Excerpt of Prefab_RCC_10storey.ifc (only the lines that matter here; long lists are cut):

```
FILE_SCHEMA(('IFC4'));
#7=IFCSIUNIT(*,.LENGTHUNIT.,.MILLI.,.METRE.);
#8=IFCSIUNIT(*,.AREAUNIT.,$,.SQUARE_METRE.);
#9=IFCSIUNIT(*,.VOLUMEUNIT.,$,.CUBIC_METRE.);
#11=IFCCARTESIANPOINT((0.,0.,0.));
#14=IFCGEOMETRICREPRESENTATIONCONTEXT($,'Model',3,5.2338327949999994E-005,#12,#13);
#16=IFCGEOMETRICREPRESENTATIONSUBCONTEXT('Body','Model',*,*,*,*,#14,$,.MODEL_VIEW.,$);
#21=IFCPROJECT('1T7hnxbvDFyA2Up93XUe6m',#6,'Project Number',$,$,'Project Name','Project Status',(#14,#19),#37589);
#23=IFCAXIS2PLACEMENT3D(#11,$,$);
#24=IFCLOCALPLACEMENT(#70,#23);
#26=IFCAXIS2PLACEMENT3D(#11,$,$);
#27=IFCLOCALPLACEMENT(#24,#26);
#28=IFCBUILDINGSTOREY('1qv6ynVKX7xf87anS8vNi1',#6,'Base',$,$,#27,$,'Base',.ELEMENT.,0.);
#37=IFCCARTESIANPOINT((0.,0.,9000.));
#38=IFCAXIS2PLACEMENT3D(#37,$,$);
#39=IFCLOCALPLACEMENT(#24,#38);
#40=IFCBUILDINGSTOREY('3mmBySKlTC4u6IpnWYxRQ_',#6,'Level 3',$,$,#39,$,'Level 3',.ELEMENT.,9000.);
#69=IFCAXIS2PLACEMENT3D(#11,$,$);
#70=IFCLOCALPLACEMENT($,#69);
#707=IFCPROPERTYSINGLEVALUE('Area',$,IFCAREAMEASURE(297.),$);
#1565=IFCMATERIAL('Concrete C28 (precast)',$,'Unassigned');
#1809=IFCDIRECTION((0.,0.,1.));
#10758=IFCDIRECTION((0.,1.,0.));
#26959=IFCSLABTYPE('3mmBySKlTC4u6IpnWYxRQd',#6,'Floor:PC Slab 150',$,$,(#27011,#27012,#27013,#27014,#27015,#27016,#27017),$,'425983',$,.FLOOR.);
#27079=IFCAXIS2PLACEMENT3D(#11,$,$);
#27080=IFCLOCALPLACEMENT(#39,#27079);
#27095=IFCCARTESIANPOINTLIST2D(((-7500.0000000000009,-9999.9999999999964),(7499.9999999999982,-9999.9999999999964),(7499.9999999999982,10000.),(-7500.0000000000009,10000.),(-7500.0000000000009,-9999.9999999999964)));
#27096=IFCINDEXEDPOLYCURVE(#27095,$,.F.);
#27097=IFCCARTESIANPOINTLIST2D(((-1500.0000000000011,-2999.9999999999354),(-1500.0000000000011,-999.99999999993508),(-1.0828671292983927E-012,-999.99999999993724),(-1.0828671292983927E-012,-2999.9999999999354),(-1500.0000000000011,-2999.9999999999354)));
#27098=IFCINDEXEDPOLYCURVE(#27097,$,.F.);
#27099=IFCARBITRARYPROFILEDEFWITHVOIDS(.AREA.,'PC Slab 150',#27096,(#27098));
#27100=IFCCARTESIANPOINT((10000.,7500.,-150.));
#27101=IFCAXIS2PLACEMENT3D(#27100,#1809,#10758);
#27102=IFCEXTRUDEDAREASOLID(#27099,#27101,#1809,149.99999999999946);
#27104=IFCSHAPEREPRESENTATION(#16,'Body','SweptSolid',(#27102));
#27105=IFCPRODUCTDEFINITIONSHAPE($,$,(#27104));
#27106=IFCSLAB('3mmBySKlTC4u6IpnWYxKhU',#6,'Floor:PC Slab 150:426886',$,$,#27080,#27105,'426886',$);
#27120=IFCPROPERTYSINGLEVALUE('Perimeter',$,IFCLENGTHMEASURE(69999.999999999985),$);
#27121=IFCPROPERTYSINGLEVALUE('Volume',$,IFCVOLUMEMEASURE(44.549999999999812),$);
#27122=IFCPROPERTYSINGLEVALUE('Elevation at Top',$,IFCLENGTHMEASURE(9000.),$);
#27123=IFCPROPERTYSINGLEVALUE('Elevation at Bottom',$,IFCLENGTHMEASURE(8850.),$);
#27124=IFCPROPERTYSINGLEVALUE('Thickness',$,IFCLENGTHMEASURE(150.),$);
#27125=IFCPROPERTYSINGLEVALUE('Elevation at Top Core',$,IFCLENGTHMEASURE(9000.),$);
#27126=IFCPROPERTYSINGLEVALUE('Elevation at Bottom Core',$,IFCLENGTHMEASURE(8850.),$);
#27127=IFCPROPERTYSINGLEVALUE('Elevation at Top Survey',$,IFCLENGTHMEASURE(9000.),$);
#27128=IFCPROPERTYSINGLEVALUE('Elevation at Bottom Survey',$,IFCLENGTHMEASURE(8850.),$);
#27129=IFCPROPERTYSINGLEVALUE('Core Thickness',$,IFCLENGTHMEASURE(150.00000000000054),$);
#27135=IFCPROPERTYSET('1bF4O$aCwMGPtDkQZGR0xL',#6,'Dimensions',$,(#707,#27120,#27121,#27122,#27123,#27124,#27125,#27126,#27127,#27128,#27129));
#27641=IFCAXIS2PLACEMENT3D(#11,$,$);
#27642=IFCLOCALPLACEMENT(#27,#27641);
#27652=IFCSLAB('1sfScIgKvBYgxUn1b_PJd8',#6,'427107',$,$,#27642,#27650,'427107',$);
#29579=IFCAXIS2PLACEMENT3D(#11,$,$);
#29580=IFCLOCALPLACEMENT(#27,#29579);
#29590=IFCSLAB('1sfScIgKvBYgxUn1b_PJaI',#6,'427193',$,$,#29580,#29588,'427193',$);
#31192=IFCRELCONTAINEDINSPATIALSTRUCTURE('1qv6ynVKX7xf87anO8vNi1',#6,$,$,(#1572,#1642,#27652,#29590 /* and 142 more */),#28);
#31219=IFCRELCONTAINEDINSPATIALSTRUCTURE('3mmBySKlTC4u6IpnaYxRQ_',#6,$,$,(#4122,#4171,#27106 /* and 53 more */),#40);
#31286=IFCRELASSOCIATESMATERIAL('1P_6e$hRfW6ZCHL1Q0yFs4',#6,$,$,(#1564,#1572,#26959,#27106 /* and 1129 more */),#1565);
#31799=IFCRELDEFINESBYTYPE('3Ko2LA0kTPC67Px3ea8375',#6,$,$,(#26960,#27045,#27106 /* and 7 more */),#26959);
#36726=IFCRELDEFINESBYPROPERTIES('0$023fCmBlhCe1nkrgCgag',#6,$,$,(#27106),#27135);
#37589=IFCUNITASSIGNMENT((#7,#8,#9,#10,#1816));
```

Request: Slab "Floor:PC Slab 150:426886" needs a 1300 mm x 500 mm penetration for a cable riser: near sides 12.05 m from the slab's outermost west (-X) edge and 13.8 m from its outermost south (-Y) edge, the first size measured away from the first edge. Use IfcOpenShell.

```python
import numpy as np
import ifcopenshell
import ifcopenshell.api.feature
import ifcopenshell.api.geometry
import ifcopenshell.api.pset
import ifcopenshell.api.root
import ifcopenshell.geom
import ifcopenshell.util.element
import ifcopenshell.util.placement
import ifcopenshell.util.representation
import ifcopenshell.util.shape
import ifcopenshell.util.unit

model = ifcopenshell.open("Prefab_RCC_10storey.ifc")
unit_scale = ifcopenshell.util.unit.calculate_unit_scale(model)
area_scale = ifcopenshell.util.unit.calculate_unit_scale(model, "AREAUNIT")
volume_scale = ifcopenshell.util.unit.calculate_unit_scale(model, "VOLUMEUNIT")
settings = ifcopenshell.geom.settings()


def volume(element):
    """Net volume in cubic metres, openings subtracted."""
    shape = ifcopenshell.geom.create_shape(settings, element)
    return ifcopenshell.util.shape.get_volume(shape.geometry)


slab = model.by_id(27106)
before = volume(slab)

# Extent in the slab's own axes, in metres. The edges named are its -X and -Y sides.
slab_shape = ifcopenshell.geom.create_shape(settings, slab)
vertices = ifcopenshell.util.shape.get_vertices(slab_shape.geometry)
x_min, y_min, bottom = vertices.min(axis=0)
top = vertices[:, 2].max()

opening = ifcopenshell.api.root.create_entity(model, ifc_class="IfcOpeningElement", name="Cable riser opening", predefined_type="OPENING")
context = ifcopenshell.util.representation.get_context(model, "Model", "Body", "MODEL_VIEW")
width, depth = 1.3, 0.5
outline = [(0.0, 0.0), (width, 0.0), (width, depth), (0.0, depth), (0.0, 0.0)]
# Overshoot both faces by 50 mm so the cut is clean.
shape = ifcopenshell.api.geometry.add_slab_representation(
    model, context=context, depth=top - bottom + 0.1, polyline=outline
)
ifcopenshell.api.geometry.assign_representation(model, product=opening, representation=shape)

matrix = ifcopenshell.util.placement.get_local_placement(slab.ObjectPlacement)
matrix[:, 3] = matrix @ np.append(np.array([x_min + 12.05, y_min + 13.8, bottom - 0.05]) / unit_scale, 1.0)
ifcopenshell.api.geometry.edit_object_placement(model, product=opening, matrix=matrix, is_si=False)
ifcopenshell.api.feature.add_feature(model, feature=opening, element=slab)

after = volume(slab)

# Update the slab's stored quantities.
pset = model.by_id(ifcopenshell.util.element.get_pset(slab, "Dimensions", should_inherit=False)["id"])
ifcopenshell.api.pset.edit_pset(model, pset=pset, properties={
    "Area": model.create_entity("IfcAreaMeasure", after / (top - bottom) / area_scale),
    "Volume": model.create_entity("IfcVolumeMeasure", after / volume_scale),
})

print(f"slab volume {before:.3f} -> {after:.3f} m3")

model.write("Prefab_RCC_10storey_updated.ifc")
```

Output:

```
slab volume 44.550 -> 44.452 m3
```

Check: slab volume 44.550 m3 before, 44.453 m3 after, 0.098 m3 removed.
